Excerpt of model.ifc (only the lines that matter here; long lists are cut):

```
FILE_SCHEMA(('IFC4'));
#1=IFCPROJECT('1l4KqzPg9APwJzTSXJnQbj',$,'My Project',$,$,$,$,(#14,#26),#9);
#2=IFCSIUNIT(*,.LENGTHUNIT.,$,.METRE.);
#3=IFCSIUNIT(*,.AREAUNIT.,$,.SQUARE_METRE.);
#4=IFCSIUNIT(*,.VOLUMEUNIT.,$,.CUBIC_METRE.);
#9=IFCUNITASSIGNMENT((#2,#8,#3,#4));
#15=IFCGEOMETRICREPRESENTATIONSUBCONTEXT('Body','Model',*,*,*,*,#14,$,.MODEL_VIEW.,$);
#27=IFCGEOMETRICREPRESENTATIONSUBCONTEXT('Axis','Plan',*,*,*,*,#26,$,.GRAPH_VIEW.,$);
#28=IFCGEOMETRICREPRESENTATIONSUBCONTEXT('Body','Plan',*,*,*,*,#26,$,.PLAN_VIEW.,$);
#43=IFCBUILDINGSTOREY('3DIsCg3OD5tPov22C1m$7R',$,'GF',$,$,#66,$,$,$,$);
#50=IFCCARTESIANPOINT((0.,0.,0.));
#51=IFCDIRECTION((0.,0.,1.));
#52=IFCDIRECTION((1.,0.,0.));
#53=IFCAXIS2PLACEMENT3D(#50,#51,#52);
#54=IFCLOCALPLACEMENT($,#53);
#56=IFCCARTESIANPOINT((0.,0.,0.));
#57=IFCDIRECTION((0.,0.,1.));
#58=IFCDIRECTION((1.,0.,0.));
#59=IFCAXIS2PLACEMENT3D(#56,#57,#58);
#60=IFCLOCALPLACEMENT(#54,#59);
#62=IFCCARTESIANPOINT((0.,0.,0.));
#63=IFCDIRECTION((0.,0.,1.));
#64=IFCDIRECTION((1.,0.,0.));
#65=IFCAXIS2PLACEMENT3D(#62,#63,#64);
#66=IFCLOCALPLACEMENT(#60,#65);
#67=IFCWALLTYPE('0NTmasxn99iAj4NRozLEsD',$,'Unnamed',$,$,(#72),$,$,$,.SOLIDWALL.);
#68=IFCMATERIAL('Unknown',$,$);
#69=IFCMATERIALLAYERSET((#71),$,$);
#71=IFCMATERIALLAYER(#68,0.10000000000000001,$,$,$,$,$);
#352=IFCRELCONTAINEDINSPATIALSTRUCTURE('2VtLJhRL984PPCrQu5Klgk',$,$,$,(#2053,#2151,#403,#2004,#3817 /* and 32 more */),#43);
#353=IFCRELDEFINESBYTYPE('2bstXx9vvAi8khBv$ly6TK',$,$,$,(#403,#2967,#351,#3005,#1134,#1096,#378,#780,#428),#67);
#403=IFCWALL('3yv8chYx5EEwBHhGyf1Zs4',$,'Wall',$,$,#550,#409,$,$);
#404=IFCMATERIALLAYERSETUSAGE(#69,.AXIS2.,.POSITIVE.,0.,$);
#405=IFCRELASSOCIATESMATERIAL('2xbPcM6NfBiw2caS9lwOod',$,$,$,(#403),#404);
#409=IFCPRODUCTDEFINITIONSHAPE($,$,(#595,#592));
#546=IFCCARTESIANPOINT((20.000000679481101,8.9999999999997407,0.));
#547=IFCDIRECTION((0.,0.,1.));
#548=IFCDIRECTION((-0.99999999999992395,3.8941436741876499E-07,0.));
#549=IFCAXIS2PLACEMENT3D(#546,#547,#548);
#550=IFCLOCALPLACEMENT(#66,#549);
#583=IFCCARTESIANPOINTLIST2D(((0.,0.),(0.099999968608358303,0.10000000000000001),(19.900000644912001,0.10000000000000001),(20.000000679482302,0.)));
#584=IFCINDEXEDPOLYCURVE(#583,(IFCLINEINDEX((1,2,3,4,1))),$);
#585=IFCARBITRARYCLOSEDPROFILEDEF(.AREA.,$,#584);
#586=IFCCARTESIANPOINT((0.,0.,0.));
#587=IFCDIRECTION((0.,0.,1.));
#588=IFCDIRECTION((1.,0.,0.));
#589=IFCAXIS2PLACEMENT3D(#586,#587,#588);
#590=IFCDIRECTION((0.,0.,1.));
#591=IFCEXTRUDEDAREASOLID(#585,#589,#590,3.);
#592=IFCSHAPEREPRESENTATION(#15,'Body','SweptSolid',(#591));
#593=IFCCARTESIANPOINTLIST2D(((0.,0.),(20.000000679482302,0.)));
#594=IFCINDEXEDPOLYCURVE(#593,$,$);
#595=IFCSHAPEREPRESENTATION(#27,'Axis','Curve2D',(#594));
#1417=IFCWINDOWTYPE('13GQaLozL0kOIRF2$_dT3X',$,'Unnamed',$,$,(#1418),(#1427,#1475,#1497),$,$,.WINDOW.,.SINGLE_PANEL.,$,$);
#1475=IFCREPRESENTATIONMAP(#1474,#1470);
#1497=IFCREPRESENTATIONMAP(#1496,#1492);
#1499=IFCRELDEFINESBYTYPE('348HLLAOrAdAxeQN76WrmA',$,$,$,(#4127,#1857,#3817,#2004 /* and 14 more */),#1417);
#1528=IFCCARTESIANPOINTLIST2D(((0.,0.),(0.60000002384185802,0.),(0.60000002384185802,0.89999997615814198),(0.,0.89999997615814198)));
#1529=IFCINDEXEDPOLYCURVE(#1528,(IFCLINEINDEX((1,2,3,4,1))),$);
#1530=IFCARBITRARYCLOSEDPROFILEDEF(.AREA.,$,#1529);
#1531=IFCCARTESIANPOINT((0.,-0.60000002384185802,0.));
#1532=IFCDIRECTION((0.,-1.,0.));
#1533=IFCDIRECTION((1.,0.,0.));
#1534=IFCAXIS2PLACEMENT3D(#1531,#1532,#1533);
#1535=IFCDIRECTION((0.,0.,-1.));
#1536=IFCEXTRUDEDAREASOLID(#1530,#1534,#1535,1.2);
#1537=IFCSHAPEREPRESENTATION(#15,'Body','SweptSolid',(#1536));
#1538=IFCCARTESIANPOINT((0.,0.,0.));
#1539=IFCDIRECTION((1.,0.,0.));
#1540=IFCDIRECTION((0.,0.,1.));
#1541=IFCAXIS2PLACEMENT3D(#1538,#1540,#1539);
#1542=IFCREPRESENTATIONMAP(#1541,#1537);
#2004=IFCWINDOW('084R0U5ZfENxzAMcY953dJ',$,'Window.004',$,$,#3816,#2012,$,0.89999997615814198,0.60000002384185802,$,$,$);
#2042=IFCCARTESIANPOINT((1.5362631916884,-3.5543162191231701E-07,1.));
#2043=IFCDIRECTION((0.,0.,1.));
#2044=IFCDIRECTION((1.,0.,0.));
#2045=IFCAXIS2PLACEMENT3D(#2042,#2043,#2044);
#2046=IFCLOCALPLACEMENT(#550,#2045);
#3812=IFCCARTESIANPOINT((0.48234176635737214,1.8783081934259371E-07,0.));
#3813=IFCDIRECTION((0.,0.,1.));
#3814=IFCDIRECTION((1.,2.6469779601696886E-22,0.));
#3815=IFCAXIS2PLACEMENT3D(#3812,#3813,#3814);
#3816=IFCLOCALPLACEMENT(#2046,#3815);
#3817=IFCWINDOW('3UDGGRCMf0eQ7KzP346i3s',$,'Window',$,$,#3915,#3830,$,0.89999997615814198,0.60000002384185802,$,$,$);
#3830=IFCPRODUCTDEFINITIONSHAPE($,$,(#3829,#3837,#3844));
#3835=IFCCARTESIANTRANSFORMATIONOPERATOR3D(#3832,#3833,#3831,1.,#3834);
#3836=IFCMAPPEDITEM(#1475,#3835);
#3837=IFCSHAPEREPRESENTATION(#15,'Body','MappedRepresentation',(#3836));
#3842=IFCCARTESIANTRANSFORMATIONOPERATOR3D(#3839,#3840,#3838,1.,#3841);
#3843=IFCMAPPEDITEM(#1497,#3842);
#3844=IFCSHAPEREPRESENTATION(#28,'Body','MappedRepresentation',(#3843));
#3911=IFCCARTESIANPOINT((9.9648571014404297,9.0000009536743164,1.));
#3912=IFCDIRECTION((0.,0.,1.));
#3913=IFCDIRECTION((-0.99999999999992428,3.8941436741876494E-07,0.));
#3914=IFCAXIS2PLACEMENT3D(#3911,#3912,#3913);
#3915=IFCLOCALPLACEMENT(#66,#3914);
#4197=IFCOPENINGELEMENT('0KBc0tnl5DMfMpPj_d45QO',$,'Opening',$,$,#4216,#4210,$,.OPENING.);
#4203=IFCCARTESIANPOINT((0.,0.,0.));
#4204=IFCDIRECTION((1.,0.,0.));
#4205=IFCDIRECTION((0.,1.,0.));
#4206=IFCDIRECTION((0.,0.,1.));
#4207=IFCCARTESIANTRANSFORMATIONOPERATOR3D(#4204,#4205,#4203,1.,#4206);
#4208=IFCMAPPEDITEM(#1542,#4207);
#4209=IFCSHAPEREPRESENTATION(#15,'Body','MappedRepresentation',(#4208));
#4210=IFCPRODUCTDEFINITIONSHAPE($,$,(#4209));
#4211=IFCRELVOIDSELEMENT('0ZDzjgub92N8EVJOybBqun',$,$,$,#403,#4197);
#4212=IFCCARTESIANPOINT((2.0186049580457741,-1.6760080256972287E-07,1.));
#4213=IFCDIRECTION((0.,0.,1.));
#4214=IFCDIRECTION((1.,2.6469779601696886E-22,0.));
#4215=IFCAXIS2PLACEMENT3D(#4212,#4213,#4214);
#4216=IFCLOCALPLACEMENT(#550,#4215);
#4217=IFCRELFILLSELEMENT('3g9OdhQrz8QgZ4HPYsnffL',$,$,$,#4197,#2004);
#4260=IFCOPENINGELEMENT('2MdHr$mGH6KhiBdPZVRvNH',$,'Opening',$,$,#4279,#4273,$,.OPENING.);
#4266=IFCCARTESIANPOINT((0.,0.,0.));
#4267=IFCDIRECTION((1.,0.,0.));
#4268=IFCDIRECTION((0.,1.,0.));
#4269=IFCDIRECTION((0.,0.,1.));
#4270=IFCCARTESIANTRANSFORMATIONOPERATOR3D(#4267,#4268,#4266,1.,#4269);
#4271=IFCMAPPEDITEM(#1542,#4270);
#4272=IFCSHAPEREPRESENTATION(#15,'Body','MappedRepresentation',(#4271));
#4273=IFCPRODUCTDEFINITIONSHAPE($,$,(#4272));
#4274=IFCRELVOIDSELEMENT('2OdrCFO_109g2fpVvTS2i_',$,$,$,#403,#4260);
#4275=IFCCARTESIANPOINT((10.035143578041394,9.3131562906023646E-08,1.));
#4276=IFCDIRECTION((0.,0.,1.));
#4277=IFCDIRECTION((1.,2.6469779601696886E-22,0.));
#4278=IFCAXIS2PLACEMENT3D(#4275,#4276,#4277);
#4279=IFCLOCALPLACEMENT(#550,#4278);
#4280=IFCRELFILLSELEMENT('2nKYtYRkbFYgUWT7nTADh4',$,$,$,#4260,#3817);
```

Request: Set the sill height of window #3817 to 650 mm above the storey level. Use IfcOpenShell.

```python
import numpy as np
import ifcopenshell
import ifcopenshell.api.geometry
import ifcopenshell.geom
import ifcopenshell.util.element
import ifcopenshell.util.placement
import ifcopenshell.util.shape
import ifcopenshell.util.unit

model = ifcopenshell.open("model.ifc")
unit_scale = ifcopenshell.util.unit.calculate_unit_scale(model)

window = model.by_guid("3UDGGRCMf0eQ7KzP346i3s")
opening = window.FillsVoids[0].RelatingOpeningElement
storey = ifcopenshell.util.element.get_container(window, ifc_class="IfcBuildingStorey")
level = ifcopenshell.util.placement.get_local_placement(storey.ObjectPlacement)[2, 3]

# The opening's origin need not be at the sill, so measure its lowest point.
shape = ifcopenshell.geom.create_shape(ifcopenshell.geom.settings(), opening)
bottom = ifcopenshell.util.shape.get_shape_bottom_elevation(shape, shape.geometry) / unit_scale
dz = level + 0.65 / unit_scale - bottom

shift = np.array([0.0, 0.0, dz])
# The window is not placed relative to its opening, so move both.
for product in (opening, window):
    matrix = ifcopenshell.util.placement.get_local_placement(product.ObjectPlacement)
    matrix[:3, 3] += shift
    ifcopenshell.api.geometry.edit_object_placement(model, product=product, matrix=matrix, is_si=False)

print(f"moved by {dz * unit_scale:+.3f} m")

model.write("model_v2.ifc")
```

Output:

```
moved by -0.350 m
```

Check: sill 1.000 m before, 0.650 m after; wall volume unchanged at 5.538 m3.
